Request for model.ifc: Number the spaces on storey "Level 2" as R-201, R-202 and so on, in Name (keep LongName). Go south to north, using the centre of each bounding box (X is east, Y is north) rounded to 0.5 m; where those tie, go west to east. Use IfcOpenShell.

First a look at what the model holds.

```python
import ifcopenshell
import ifcopenshell.util.element
import ifcopenshell.util.placement

model = ifcopenshell.open("model.ifc")
print(model.schema)
storey = next(s for s in model.by_type("IfcBuildingStorey") if s.Name == "Level 2")
spaces = [e for e in ifcopenshell.util.element.get_decomposition(storey) if e.is_a("IfcSpace")]
for e in sorted(spaces, key=lambda e: e.id()):
    origin = ifcopenshell.util.placement.get_local_placement(e.ObjectPlacement)[:3, 3]
    print(e.id(), e.Name, e.LongName, origin.round(2) + 0.0, sep=" | ")
```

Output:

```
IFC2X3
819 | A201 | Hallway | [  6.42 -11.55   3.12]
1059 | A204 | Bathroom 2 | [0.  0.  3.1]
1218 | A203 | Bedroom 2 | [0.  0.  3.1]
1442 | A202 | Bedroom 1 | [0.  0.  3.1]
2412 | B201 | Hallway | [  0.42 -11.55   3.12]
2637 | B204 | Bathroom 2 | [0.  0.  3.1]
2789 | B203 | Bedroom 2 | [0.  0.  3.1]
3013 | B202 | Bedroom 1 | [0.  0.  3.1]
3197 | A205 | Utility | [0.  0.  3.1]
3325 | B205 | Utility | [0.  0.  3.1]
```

```python
import ifcopenshell
import ifcopenshell.geom
import ifcopenshell.util.element
import ifcopenshell.util.shape

model = ifcopenshell.open("model.ifc")
settings = ifcopenshell.geom.settings()
settings.set("use-world-coords", True)


def centre(element):
    shape = ifcopenshell.geom.create_shape(settings, element)
    return ifcopenshell.util.shape.get_bbox_centroid(shape.geometry)


storey = next(s for s in model.by_type("IfcBuildingStorey") if s.Name == "Level 2")
spaces = [e for e in ifcopenshell.util.element.get_decomposition(storey) if e.is_a("IfcSpace")]

# Insertion points can sit at a corner or the storey origin, so sort by the geometry (in metres).
centres = {e: centre(e) for e in spaces}
spaces.sort(key=lambda e: (round(centres[e][1] / 0.5), centres[e][0]))

for i, e in enumerate(spaces, start=1):
    number = f"R-2{i:02d}"
    e.Name = number
    print(e.id(), number)

model.write("model_edited.ifc")
```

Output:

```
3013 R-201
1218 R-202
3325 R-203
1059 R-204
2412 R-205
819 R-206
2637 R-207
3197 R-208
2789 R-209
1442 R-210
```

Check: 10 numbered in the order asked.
